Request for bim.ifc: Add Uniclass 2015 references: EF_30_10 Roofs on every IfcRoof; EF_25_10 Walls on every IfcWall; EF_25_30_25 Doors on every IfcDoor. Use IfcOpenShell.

First a look at what the model holds.

```python
import ifcopenshell

model = ifcopenshell.open("bim.ifc")
print(model.schema)
print("classifications:", [c.Name for c in model.by_type("IfcClassification")])
for ifc_class in ("IfcDoor", "IfcRoof", "IfcStair", "IfcWall", "IfcWindow"):
    print(ifc_class, len(model.by_type(ifc_class)))
```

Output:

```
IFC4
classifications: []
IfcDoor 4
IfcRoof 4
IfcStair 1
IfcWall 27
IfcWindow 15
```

```python
import ifcopenshell
import ifcopenshell.api.classification

model = ifcopenshell.open("bim.ifc")

system = ifcopenshell.api.classification.add_classification(model, classification="Uniclass 2015")

codes = {
    "IfcRoof": ("EF_30_10", "Roofs"),
    "IfcWall": ("EF_25_10", "Walls"),
    "IfcDoor": ("EF_25_30_25", "Doors"),
}
for ifc_class, (code, name) in codes.items():
    products = model.by_type(ifc_class)
    ifcopenshell.api.classification.add_reference(
        model, products=products, classification=system, identification=code, name=name
    )
    print(code, len(products))

model.write("bim-out.ifc")
```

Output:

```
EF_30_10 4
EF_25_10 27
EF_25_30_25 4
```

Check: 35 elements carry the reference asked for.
